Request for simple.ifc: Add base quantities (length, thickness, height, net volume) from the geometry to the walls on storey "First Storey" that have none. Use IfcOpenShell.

First a look at what the model holds.

```python
import ifcopenshell
import ifcopenshell.util.element
import ifcopenshell.util.unit

model = ifcopenshell.open("simple.ifc")
print(model.schema)
for unit_type in ("LENGTHUNIT", "AREAUNIT", "VOLUMEUNIT"):
    print(unit_type, ifcopenshell.util.unit.calculate_unit_scale(model, unit_type))
storey = next(s for s in model.by_type("IfcBuildingStorey") if s.Name == "First Storey")
walls = [e for e in ifcopenshell.util.element.get_decomposition(storey) if e.is_a("IfcWall")]
for e in sorted(walls, key=lambda e: e.id()):
    print(e.id(), e.is_a(), e.Name, list(ifcopenshell.util.element.get_psets(e, qtos_only=True)), sep=" | ")
```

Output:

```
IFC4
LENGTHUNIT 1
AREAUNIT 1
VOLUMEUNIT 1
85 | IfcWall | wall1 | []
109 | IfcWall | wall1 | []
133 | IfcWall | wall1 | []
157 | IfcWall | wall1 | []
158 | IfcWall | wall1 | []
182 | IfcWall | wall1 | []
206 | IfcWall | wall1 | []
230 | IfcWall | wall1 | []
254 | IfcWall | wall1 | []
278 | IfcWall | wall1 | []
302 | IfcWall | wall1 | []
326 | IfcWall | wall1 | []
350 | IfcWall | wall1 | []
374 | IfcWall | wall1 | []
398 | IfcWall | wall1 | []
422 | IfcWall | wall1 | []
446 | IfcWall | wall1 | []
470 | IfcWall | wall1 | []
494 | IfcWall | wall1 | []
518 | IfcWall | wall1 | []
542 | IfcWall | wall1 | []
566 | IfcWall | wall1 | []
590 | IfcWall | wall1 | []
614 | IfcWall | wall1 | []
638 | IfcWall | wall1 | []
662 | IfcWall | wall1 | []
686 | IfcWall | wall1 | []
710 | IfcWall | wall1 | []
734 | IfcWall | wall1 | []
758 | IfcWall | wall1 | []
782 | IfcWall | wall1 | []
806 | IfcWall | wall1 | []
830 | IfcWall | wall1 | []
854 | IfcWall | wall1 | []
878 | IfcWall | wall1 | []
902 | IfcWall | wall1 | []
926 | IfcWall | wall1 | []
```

```python
import ifcopenshell
import ifcopenshell.api.pset
import ifcopenshell.geom
import ifcopenshell.util.element
import ifcopenshell.util.shape
import ifcopenshell.util.unit

model = ifcopenshell.open("simple.ifc")
unit_scale = ifcopenshell.util.unit.calculate_unit_scale(model)
volume_scale = ifcopenshell.util.unit.calculate_unit_scale(model, "VOLUMEUNIT")
settings = ifcopenshell.geom.settings()

storey = next(s for s in model.by_type("IfcBuildingStorey") if s.Name == "First Storey")
walls = [e for e in ifcopenshell.util.element.get_decomposition(storey) if e.is_a("IfcWall")]

for e in sorted(walls, key=lambda e: e.id()):
    if ifcopenshell.util.element.get_psets(e, qtos_only=True, should_inherit=False):
        continue
    # Geometry comes back in metres, in the element's own axes.
    shape = ifcopenshell.geom.create_shape(settings, e)
    values = {
        "Length": ifcopenshell.util.shape.get_x(shape.geometry) / unit_scale,
        "Width": ifcopenshell.util.shape.get_y(shape.geometry) / unit_scale,
        "Height": ifcopenshell.util.shape.get_z(shape.geometry) / unit_scale,
        "NetVolume": ifcopenshell.util.shape.get_volume(shape.geometry) / volume_scale,
    }
    qto = ifcopenshell.api.pset.add_qto(model, product=e, name="Qto_WallBaseQuantities")
    ifcopenshell.api.pset.edit_qto(model, qto=qto, properties=values)
    print(e.id(), {k: round(v, 3) for k, v in values.items()})

model.write("simple_rev.ifc")
```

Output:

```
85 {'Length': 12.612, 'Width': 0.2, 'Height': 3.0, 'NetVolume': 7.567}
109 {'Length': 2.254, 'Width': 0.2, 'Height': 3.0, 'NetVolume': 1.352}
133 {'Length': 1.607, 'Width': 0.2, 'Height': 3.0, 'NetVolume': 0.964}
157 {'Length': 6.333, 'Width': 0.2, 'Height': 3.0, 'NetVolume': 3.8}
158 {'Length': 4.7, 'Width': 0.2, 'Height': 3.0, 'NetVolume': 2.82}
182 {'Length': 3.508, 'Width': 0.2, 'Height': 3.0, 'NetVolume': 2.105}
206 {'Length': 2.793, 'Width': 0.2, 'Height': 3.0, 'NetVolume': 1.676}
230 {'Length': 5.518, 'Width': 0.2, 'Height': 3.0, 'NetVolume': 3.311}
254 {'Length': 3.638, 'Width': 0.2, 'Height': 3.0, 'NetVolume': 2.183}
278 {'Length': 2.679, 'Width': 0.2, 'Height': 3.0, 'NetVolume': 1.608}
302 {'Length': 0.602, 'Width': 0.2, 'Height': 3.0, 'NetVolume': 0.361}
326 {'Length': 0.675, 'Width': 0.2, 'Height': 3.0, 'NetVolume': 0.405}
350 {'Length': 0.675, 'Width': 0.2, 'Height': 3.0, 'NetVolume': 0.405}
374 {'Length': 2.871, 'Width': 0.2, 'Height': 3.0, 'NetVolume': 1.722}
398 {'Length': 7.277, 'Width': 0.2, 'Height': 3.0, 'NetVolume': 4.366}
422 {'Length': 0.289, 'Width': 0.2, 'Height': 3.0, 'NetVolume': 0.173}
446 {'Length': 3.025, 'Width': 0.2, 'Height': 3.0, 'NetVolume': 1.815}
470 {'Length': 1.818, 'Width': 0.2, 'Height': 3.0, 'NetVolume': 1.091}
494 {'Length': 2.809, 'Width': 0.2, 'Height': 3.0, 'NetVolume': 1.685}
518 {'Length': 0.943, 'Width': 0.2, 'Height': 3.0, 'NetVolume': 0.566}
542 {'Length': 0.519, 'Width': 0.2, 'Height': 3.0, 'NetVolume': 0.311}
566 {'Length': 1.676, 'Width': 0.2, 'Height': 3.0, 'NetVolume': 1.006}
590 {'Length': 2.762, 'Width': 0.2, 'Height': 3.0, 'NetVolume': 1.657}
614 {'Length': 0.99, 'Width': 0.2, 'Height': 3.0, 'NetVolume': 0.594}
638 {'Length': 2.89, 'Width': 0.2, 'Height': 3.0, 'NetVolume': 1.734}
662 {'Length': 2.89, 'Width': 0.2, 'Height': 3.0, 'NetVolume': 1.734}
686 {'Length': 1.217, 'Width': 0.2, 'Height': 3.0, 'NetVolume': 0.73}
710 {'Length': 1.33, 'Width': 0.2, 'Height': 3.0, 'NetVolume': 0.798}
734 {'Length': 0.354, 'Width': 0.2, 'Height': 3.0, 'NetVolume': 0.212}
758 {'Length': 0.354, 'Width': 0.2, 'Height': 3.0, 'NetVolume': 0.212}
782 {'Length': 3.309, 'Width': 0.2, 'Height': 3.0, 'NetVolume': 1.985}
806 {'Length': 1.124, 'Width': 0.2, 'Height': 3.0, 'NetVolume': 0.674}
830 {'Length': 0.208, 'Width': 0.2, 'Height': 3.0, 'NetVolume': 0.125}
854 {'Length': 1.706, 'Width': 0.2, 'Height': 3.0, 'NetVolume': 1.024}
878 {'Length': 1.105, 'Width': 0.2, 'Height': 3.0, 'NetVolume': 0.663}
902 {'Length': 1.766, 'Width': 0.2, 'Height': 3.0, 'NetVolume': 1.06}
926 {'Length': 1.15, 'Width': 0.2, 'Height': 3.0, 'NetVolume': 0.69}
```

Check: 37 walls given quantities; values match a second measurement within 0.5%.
